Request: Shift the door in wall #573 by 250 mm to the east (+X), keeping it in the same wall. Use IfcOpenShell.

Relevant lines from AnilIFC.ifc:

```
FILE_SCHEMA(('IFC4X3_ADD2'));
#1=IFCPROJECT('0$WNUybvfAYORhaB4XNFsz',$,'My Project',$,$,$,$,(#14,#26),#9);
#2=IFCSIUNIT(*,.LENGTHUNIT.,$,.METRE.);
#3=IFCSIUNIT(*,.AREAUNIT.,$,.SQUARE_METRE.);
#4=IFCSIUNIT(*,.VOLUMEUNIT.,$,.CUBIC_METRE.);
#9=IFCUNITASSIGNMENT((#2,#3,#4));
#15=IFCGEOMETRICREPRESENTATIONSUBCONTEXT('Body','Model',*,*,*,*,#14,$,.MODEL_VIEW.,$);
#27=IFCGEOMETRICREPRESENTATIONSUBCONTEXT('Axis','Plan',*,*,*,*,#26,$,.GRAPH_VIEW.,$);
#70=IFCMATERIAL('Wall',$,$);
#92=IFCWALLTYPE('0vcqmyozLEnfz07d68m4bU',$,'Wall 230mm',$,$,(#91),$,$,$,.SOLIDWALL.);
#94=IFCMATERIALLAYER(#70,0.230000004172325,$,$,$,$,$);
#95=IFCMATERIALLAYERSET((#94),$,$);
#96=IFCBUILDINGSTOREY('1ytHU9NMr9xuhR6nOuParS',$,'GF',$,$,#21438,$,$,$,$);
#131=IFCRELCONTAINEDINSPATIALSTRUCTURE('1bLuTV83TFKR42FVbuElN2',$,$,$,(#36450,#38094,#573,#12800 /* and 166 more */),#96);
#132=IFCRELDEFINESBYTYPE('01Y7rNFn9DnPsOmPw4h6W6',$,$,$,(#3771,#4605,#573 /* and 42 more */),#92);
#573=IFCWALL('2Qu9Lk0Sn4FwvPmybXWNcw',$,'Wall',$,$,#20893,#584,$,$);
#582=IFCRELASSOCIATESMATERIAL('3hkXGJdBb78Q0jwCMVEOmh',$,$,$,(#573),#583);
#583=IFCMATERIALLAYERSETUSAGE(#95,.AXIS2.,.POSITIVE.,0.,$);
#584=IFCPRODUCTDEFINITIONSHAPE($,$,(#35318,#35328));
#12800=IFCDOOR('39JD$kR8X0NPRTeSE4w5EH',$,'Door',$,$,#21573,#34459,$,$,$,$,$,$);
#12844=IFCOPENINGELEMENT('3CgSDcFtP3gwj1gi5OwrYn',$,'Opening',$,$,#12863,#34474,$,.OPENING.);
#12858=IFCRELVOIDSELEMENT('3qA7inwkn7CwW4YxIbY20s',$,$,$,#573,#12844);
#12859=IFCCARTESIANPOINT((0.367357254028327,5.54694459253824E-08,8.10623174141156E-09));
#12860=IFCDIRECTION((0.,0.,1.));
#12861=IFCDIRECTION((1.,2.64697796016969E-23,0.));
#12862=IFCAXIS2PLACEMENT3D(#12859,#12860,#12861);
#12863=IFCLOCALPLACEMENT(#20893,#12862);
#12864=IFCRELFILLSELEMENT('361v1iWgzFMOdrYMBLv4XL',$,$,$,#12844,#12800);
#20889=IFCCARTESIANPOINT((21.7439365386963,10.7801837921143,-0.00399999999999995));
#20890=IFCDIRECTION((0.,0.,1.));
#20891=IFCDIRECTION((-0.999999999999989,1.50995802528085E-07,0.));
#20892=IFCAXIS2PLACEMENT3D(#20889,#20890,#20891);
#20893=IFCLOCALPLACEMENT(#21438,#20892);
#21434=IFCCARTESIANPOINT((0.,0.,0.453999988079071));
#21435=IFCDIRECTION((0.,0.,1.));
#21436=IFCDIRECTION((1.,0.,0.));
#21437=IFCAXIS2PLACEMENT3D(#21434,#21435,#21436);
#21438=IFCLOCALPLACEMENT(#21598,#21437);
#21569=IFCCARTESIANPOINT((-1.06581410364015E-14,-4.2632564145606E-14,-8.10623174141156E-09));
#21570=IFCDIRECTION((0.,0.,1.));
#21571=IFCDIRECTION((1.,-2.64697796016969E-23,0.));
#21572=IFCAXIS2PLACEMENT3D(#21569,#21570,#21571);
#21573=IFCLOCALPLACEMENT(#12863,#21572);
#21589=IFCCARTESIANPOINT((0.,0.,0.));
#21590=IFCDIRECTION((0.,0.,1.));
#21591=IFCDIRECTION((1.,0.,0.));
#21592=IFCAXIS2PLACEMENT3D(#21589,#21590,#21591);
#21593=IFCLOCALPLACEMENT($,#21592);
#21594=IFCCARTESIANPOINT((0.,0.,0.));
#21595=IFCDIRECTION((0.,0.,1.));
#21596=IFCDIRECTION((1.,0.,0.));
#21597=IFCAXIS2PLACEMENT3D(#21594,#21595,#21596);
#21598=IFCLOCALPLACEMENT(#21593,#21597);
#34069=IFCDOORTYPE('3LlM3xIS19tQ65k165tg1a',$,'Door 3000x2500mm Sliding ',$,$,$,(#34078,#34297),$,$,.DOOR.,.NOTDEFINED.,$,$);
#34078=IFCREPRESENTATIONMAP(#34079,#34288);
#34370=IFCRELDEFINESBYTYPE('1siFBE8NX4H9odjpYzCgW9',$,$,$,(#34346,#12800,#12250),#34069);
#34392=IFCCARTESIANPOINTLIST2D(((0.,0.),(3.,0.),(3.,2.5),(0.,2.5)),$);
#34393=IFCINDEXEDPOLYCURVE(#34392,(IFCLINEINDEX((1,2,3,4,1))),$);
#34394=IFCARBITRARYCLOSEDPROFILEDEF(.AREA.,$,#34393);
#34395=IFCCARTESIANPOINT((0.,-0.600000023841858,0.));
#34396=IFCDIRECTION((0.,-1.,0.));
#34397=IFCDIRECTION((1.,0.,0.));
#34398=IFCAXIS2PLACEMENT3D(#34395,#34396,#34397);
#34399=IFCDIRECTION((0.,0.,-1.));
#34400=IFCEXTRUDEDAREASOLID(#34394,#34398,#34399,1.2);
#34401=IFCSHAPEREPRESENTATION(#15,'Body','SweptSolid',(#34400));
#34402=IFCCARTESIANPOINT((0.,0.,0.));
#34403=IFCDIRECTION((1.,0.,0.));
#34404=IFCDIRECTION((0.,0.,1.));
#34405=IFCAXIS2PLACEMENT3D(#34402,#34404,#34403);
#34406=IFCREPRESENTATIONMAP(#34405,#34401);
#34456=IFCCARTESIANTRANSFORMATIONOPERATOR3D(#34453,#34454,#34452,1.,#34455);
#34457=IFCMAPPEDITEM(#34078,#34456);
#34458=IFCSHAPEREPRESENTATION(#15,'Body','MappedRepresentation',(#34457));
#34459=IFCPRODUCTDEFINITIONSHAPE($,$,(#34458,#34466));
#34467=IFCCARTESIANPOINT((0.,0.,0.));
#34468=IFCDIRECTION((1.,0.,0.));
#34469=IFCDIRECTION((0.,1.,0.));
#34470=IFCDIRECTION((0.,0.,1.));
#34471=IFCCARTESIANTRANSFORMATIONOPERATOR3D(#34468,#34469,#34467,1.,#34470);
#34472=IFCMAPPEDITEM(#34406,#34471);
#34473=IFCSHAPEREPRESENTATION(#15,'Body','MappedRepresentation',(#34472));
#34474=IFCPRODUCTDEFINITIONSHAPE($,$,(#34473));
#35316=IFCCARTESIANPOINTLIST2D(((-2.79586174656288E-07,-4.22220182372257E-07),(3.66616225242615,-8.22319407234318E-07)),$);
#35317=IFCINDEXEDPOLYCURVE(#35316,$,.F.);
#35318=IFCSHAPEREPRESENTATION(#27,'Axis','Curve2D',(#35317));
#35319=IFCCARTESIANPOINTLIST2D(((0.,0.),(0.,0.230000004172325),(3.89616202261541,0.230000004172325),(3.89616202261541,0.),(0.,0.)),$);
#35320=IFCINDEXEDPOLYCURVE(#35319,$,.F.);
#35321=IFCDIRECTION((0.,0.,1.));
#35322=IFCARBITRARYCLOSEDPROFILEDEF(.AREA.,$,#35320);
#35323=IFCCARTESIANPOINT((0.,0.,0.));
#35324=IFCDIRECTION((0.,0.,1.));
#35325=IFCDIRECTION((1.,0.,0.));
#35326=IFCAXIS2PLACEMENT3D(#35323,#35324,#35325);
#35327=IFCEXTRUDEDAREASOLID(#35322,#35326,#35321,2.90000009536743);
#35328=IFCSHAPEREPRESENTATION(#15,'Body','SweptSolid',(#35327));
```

```python
import ifcopenshell
import ifcopenshell.api.geometry
import ifcopenshell.util.placement
import ifcopenshell.util.unit

model = ifcopenshell.open("AnilIFC.ifc")
unit_scale = ifcopenshell.util.unit.calculate_unit_scale(model)

door = model.by_id(12800)
opening = door.FillsVoids[0].RelatingOpeningElement
wall = opening.VoidsElements[0].RelatingBuildingElement

wall_matrix = ifcopenshell.util.placement.get_local_placement(wall.ObjectPlacement)
shift = wall_matrix[:3, 0] * -0.25 / unit_scale
before = ifcopenshell.util.placement.get_local_placement(door.ObjectPlacement)[:3, 3].copy()

# The door is placed relative to its opening, so it follows when the opening moves.
matrix = ifcopenshell.util.placement.get_local_placement(opening.ObjectPlacement)
matrix[:3, 3] += shift
ifcopenshell.api.geometry.edit_object_placement(
    model, product=opening, matrix=matrix, is_si=False, should_transform_children=True
)

after = ifcopenshell.util.placement.get_local_placement(door.ObjectPlacement)[:3, 3]
print("door moved by", (after - before).round(3) + 0.0)

model.write("AnilIFC-out.ifc")
```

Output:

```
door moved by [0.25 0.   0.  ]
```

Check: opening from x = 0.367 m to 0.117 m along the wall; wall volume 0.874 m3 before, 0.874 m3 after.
